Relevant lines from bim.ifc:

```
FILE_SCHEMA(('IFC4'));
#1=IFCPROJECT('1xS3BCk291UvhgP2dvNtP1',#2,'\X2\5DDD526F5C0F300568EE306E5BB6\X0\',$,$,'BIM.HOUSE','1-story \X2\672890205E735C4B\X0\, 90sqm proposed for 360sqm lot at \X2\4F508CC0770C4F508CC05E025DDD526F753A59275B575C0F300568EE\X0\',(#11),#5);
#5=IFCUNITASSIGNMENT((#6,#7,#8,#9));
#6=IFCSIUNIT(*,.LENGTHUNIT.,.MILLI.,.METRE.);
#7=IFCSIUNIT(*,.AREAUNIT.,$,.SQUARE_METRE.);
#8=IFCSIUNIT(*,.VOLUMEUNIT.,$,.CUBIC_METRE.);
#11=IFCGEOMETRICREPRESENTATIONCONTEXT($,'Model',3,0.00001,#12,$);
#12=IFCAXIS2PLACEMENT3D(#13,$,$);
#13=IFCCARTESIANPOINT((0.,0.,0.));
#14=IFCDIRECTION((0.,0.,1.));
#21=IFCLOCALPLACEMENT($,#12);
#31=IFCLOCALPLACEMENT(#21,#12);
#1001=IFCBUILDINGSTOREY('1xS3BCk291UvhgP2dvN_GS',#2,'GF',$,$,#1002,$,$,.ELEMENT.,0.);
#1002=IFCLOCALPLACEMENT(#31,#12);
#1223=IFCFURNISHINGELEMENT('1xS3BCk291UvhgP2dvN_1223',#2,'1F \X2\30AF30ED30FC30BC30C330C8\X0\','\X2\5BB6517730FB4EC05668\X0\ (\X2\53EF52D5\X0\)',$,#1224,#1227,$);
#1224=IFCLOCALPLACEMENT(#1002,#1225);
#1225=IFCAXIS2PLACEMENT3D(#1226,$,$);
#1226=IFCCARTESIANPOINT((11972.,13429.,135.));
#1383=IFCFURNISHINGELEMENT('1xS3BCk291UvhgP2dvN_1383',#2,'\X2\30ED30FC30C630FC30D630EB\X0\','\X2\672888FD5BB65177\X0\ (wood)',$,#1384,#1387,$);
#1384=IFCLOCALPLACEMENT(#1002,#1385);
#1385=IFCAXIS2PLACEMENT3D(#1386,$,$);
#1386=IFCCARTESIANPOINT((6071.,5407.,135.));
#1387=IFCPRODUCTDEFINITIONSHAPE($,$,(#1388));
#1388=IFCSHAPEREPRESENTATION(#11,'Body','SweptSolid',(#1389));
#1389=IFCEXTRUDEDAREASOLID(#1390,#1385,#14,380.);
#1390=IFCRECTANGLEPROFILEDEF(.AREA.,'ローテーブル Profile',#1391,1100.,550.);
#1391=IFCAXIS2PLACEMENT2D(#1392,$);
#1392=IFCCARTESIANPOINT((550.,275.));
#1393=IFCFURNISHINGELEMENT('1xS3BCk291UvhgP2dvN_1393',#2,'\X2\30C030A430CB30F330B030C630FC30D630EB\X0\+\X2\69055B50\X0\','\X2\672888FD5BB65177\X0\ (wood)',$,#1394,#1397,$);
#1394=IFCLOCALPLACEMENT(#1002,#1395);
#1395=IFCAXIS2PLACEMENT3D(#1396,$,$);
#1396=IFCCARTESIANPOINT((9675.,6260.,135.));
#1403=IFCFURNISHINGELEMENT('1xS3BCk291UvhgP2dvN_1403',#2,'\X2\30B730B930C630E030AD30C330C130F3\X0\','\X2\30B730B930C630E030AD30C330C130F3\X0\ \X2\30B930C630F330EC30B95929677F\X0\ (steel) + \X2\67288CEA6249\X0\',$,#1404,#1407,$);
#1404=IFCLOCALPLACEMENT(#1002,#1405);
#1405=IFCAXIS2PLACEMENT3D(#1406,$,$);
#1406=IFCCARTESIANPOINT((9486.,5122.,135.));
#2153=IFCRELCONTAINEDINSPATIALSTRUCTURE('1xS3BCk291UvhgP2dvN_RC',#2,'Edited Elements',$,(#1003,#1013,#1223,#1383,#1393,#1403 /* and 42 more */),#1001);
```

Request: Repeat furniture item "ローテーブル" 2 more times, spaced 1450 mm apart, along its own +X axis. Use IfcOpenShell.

```python
import ifcopenshell
import ifcopenshell.api.geometry
import ifcopenshell.api.root
import ifcopenshell.util.element
import ifcopenshell.util.placement

model = ifcopenshell.open("bim.ifc")


def reuse_history(source, copy):
    """copy_class also copies each property set's owner history, people and application; keep the originals."""
    for rel in copy.IsDefinedBy:
        if rel.is_a("IfcRelDefinesByProperties") and (history := rel.RelatingPropertyDefinition.OwnerHistory):
            rel.RelatingPropertyDefinition.OwnerHistory = source.OwnerHistory
            ifcopenshell.util.element.remove_deep2(model, history)


source = model.by_guid("1xS3BCk291UvhgP2dvN_1383")
base = ifcopenshell.util.placement.get_local_placement(source.ObjectPlacement)
step = base[:3, 0] * 1450.0

for i in range(1, 3):
    copy = ifcopenshell.api.root.copy_class(model, product=source)
    copy.Representation = ifcopenshell.util.element.copy_deep(
        model, source.Representation, exclude=["IfcGeometricRepresentationContext", "IfcRepresentationMap"]
    )
    reuse_history(source, copy)
    matrix = base.copy()
    matrix[:3, 3] += i * step
    print("added at", matrix[:3, 3].round(3) + 0.0)
    ifcopenshell.api.geometry.edit_object_placement(model, product=copy, matrix=matrix, is_si=False)

model.write("bim_v2.ifc")
```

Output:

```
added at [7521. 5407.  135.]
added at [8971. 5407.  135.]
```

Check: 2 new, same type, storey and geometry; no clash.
